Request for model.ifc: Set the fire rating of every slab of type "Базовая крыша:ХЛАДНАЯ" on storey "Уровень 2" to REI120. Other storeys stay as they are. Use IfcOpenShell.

First a look at what the model holds.

```python
import ifcopenshell
import ifcopenshell.util.element

model = ifcopenshell.open("model.ifc")
print(model.schema)
storey = next(s for s in model.by_type("IfcBuildingStorey") if s.Name == "Уровень 2")
slabs = [e for e in ifcopenshell.util.element.get_decomposition(storey) if e.is_a("IfcSlab")]
seen = {}
for e in slabs:
    element_type = ifcopenshell.util.element.get_type(e)
    key = (element_type.Name if element_type != e and element_type else None, ifcopenshell.util.element.get_pset(e, "Pset_SlabCommon", "FireRating"))
    seen[key] = seen.get(key, 0) + 1
for (name, value), count in sorted(seen.items(), key=str):
    print(count, "x", name, "|", value)
```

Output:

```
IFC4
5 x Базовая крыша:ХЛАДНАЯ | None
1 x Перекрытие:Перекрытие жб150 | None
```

```python
import ifcopenshell
import ifcopenshell.api.pset
import ifcopenshell.util.element

model = ifcopenshell.open("model.ifc")

storey = next(s for s in model.by_type("IfcBuildingStorey") if s.Name == "Уровень 2")
slabs = [e for e in ifcopenshell.util.element.get_decomposition(storey) if e.is_a("IfcSlab")]

count = 0
for e in slabs:
    element_type = ifcopenshell.util.element.get_type(e)
    if element_type in (None, e) or element_type.Name != "Базовая крыша:ХЛАДНАЯ":
        continue
    # add_pset returns the element's existing set when there is one.
    pset = ifcopenshell.api.pset.add_pset(model, product=e, name="Pset_SlabCommon")
    ifcopenshell.api.pset.edit_pset(model, pset=pset, properties={"FireRating": "REI120"})
    count += 1

print(count, "slabs updated")

model.write("model_edited.ifc")
```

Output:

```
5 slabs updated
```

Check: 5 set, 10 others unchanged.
